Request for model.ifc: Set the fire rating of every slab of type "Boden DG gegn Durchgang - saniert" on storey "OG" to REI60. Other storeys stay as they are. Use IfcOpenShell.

First a look at what the model holds.

```python
import ifcopenshell
import ifcopenshell.util.element

model = ifcopenshell.open("model.ifc")
print(model.schema)
storey = next(s for s in model.by_type("IfcBuildingStorey") if s.Name == "OG")
slabs = [e for e in ifcopenshell.util.element.get_decomposition(storey) if e.is_a("IfcSlab")]
seen = {}
for e in slabs:
    element_type = ifcopenshell.util.element.get_type(e)
    key = (element_type.Name if element_type != e and element_type else None, ifcopenshell.util.element.get_pset(e, "Pset_SlabCommon", "FireRating"))
    seen[key] = seen.get(key, 0) + 1
for (name, value), count in sorted(seen.items(), key=str):
    print(count, "x", name, "|", value)
```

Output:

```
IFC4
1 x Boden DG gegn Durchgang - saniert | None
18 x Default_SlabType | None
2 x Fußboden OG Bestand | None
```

```python
import ifcopenshell
import ifcopenshell.api.pset
import ifcopenshell.util.element

model = ifcopenshell.open("model.ifc")

storey = next(s for s in model.by_type("IfcBuildingStorey") if s.Name == "OG")
slabs = [e for e in ifcopenshell.util.element.get_decomposition(storey) if e.is_a("IfcSlab")]

count = 0
for e in slabs:
    element_type = ifcopenshell.util.element.get_type(e)
    if element_type in (None, e) or element_type.Name != "Boden DG gegn Durchgang - saniert":
        continue
    # add_pset returns the element's existing set when there is one.
    pset = ifcopenshell.api.pset.add_pset(model, product=e, name="Pset_SlabCommon")
    ifcopenshell.api.pset.edit_pset(model, pset=pset, properties={"FireRating": "REI60"})
    count += 1

print(count, "slabs updated")

model.write("model-out.ifc")
```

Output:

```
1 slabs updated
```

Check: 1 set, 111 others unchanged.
